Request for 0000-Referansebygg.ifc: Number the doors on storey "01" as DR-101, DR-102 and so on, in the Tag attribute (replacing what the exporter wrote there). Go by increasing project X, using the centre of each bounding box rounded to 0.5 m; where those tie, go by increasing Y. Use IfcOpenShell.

First a look at what the model holds.

```python
import ifcopenshell
import ifcopenshell.util.element
import ifcopenshell.util.placement

model = ifcopenshell.open("0000-Referansebygg.ifc")
print(model.schema)
storey = next(s for s in model.by_type("IfcBuildingStorey") if s.Name == "01")
doors = [e for e in ifcopenshell.util.element.get_decomposition(storey) if e.is_a("IfcDoor")]
for e in sorted(doors, key=lambda e: e.id()):
    origin = ifcopenshell.util.placement.get_local_placement(e.ObjectPlacement)[:3, 3]
    print(e.id(), e.Tag, e.Name, origin.round(2) + 0.0, sep=" | ")
```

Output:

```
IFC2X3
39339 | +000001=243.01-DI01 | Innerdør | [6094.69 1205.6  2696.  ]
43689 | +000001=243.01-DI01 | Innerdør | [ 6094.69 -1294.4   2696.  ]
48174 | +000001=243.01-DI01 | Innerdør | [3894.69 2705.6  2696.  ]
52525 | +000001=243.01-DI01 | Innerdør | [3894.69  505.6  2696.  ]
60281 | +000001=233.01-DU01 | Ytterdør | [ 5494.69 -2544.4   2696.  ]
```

```python
import ifcopenshell
import ifcopenshell.geom
import ifcopenshell.util.element
import ifcopenshell.util.shape

model = ifcopenshell.open("0000-Referansebygg.ifc")
settings = ifcopenshell.geom.settings()
settings.set("use-world-coords", True)


def centre(element):
    shape = ifcopenshell.geom.create_shape(settings, element)
    return ifcopenshell.util.shape.get_bbox_centroid(shape.geometry)


storey = next(s for s in model.by_type("IfcBuildingStorey") if s.Name == "01")
doors = [e for e in ifcopenshell.util.element.get_decomposition(storey) if e.is_a("IfcDoor")]

# Insertion points can sit at a corner or the storey origin, so sort by the geometry (in metres).
centres = {e: centre(e) for e in doors}
doors.sort(key=lambda e: (round(centres[e][0] / 0.5), centres[e][1]))

for i, e in enumerate(doors, start=1):
    number = f"DR-1{i:02d}"
    e.Tag = number
    print(e.id(), number)

model.write("0000-Referansebygg_updated.ifc")
```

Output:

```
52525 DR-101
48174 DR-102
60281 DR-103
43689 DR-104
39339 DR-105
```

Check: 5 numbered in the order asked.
